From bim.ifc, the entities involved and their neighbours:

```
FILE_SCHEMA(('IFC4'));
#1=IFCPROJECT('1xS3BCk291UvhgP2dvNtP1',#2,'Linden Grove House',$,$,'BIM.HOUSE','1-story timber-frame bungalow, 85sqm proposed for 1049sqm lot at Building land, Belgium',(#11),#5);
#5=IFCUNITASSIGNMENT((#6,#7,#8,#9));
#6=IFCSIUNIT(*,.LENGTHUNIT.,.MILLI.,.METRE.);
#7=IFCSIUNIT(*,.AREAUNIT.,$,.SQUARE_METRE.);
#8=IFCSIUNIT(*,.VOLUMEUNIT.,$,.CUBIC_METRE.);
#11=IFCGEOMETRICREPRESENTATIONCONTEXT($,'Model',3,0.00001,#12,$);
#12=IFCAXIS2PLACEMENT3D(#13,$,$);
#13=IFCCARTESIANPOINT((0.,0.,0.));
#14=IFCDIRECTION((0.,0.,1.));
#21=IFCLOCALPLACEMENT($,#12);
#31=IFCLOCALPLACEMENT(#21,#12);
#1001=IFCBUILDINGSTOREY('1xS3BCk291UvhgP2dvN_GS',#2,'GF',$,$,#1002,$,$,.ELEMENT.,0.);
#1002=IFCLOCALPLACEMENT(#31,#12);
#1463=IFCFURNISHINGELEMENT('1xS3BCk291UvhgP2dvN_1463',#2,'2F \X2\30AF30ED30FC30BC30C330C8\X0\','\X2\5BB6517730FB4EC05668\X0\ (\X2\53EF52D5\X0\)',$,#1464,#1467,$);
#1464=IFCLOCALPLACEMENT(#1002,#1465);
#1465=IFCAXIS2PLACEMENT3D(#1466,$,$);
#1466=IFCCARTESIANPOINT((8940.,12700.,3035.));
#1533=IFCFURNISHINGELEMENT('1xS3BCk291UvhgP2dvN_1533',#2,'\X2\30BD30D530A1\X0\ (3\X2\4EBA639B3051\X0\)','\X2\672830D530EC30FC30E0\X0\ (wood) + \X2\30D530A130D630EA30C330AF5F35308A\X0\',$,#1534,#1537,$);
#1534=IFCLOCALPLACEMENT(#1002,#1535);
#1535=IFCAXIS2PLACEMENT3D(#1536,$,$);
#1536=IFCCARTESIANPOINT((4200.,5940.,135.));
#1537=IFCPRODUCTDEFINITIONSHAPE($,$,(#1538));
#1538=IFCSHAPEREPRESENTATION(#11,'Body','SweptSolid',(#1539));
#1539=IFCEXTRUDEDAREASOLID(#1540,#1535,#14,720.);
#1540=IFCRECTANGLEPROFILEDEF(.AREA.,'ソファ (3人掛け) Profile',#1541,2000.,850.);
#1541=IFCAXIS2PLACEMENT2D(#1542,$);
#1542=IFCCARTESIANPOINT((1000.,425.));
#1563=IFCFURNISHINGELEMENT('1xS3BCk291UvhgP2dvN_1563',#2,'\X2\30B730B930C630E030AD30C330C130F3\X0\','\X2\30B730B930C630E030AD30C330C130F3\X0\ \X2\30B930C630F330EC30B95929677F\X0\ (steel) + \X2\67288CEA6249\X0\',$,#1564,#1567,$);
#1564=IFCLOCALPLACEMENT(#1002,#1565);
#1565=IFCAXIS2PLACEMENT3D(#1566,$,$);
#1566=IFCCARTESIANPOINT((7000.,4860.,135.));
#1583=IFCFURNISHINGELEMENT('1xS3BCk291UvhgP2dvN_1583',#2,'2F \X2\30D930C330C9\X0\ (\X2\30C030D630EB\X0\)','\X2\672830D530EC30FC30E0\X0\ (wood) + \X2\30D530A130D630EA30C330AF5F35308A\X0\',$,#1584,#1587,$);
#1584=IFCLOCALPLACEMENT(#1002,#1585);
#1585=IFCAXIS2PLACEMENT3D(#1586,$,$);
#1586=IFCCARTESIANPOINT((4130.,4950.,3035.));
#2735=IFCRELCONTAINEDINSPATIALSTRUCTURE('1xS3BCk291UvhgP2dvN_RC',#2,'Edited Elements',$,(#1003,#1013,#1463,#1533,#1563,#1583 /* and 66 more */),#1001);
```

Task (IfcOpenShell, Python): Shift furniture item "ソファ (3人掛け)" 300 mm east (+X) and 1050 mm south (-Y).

```python
import ifcopenshell
import ifcopenshell.api.geometry
import ifcopenshell.util.placement

model = ifcopenshell.open("bim.ifc")

item = model.by_id(1533)
matrix = ifcopenshell.util.placement.get_local_placement(item.ObjectPlacement)
matrix[0, 3] += 300.0
matrix[1, 3] -= 1050.0
ifcopenshell.api.geometry.edit_object_placement(model, product=item, matrix=matrix, is_si=False)

print(ifcopenshell.util.placement.get_local_placement(item.ObjectPlacement).round(3) + 0.0)

model.write("bim_updated.ifc")
```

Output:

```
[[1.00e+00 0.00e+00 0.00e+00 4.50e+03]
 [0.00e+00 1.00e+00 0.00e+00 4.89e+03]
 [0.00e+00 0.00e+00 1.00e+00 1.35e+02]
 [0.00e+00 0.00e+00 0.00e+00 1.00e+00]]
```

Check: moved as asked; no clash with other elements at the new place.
